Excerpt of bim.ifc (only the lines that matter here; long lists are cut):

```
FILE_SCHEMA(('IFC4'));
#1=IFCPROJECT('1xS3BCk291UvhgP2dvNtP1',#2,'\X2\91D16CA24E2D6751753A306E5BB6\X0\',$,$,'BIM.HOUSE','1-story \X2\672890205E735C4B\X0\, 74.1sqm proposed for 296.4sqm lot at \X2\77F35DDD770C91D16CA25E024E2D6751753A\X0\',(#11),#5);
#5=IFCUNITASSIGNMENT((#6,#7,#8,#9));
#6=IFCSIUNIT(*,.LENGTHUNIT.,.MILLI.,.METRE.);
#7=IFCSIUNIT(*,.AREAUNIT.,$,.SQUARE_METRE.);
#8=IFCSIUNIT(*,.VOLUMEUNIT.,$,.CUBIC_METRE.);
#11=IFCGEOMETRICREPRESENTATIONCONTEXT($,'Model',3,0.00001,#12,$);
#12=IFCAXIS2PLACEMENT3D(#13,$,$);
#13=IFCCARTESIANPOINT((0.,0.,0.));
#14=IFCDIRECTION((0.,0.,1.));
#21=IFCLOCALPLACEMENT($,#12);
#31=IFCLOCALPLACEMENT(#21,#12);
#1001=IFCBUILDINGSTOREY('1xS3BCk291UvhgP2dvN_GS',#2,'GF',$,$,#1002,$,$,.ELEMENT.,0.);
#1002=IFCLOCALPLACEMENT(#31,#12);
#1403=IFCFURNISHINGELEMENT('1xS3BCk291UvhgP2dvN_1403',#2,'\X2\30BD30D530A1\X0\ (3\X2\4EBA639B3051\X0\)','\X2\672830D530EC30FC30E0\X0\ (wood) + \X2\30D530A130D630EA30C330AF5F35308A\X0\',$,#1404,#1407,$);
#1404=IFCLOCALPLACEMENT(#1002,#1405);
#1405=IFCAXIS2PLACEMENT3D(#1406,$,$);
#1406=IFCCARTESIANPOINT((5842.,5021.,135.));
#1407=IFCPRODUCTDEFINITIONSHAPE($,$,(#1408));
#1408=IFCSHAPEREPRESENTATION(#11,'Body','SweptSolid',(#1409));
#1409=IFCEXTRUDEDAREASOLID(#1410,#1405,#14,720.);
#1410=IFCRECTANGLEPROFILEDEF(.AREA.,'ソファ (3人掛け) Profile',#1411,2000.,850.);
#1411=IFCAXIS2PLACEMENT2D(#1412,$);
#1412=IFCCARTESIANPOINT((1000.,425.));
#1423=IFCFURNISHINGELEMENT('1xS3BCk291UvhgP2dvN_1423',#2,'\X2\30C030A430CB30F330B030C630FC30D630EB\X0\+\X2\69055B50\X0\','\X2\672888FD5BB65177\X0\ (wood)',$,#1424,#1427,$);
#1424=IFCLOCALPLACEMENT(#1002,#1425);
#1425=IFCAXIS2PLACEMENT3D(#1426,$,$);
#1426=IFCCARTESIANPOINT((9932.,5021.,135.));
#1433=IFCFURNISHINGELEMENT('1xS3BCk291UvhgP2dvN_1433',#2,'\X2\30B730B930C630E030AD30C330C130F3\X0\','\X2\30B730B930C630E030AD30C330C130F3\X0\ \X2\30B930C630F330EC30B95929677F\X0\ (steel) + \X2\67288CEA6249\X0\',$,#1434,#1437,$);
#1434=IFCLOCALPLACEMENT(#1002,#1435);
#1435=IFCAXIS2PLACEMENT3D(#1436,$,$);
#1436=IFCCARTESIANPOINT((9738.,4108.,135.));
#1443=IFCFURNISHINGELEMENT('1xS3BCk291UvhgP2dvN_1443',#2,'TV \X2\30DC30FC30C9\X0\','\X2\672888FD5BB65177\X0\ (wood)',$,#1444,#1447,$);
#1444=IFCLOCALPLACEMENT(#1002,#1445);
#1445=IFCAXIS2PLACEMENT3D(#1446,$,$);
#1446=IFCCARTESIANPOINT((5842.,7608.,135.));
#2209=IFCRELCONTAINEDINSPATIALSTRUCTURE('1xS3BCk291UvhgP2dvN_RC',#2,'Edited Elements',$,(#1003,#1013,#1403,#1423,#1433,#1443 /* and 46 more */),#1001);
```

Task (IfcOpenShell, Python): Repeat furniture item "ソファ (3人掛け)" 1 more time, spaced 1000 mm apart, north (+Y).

```python
import numpy as np
import ifcopenshell
import ifcopenshell.api.geometry
import ifcopenshell.api.root
import ifcopenshell.util.element
import ifcopenshell.util.placement

model = ifcopenshell.open("bim.ifc")


def reuse_history(source, copy):
    """copy_class also copies each property set's owner history, people and application; keep the originals."""
    for rel in copy.IsDefinedBy:
        if rel.is_a("IfcRelDefinesByProperties") and (history := rel.RelatingPropertyDefinition.OwnerHistory):
            rel.RelatingPropertyDefinition.OwnerHistory = source.OwnerHistory
            ifcopenshell.util.element.remove_deep2(model, history)


source = model.by_guid("1xS3BCk291UvhgP2dvN_1403")
base = ifcopenshell.util.placement.get_local_placement(source.ObjectPlacement)
step = np.array([0.0, 1.0, 0.0]) * 1000.0

for i in range(1, 2):
    copy = ifcopenshell.api.root.copy_class(model, product=source)
    copy.Representation = ifcopenshell.util.element.copy_deep(
        model, source.Representation, exclude=["IfcGeometricRepresentationContext", "IfcRepresentationMap"]
    )
    reuse_history(source, copy)
    matrix = base.copy()
    matrix[:3, 3] += i * step
    print("added at", matrix[:3, 3].round(3) + 0.0)
    ifcopenshell.api.geometry.edit_object_placement(model, product=copy, matrix=matrix, is_si=False)

model.write("bim_edited.ifc")
```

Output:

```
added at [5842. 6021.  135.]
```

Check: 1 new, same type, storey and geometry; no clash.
